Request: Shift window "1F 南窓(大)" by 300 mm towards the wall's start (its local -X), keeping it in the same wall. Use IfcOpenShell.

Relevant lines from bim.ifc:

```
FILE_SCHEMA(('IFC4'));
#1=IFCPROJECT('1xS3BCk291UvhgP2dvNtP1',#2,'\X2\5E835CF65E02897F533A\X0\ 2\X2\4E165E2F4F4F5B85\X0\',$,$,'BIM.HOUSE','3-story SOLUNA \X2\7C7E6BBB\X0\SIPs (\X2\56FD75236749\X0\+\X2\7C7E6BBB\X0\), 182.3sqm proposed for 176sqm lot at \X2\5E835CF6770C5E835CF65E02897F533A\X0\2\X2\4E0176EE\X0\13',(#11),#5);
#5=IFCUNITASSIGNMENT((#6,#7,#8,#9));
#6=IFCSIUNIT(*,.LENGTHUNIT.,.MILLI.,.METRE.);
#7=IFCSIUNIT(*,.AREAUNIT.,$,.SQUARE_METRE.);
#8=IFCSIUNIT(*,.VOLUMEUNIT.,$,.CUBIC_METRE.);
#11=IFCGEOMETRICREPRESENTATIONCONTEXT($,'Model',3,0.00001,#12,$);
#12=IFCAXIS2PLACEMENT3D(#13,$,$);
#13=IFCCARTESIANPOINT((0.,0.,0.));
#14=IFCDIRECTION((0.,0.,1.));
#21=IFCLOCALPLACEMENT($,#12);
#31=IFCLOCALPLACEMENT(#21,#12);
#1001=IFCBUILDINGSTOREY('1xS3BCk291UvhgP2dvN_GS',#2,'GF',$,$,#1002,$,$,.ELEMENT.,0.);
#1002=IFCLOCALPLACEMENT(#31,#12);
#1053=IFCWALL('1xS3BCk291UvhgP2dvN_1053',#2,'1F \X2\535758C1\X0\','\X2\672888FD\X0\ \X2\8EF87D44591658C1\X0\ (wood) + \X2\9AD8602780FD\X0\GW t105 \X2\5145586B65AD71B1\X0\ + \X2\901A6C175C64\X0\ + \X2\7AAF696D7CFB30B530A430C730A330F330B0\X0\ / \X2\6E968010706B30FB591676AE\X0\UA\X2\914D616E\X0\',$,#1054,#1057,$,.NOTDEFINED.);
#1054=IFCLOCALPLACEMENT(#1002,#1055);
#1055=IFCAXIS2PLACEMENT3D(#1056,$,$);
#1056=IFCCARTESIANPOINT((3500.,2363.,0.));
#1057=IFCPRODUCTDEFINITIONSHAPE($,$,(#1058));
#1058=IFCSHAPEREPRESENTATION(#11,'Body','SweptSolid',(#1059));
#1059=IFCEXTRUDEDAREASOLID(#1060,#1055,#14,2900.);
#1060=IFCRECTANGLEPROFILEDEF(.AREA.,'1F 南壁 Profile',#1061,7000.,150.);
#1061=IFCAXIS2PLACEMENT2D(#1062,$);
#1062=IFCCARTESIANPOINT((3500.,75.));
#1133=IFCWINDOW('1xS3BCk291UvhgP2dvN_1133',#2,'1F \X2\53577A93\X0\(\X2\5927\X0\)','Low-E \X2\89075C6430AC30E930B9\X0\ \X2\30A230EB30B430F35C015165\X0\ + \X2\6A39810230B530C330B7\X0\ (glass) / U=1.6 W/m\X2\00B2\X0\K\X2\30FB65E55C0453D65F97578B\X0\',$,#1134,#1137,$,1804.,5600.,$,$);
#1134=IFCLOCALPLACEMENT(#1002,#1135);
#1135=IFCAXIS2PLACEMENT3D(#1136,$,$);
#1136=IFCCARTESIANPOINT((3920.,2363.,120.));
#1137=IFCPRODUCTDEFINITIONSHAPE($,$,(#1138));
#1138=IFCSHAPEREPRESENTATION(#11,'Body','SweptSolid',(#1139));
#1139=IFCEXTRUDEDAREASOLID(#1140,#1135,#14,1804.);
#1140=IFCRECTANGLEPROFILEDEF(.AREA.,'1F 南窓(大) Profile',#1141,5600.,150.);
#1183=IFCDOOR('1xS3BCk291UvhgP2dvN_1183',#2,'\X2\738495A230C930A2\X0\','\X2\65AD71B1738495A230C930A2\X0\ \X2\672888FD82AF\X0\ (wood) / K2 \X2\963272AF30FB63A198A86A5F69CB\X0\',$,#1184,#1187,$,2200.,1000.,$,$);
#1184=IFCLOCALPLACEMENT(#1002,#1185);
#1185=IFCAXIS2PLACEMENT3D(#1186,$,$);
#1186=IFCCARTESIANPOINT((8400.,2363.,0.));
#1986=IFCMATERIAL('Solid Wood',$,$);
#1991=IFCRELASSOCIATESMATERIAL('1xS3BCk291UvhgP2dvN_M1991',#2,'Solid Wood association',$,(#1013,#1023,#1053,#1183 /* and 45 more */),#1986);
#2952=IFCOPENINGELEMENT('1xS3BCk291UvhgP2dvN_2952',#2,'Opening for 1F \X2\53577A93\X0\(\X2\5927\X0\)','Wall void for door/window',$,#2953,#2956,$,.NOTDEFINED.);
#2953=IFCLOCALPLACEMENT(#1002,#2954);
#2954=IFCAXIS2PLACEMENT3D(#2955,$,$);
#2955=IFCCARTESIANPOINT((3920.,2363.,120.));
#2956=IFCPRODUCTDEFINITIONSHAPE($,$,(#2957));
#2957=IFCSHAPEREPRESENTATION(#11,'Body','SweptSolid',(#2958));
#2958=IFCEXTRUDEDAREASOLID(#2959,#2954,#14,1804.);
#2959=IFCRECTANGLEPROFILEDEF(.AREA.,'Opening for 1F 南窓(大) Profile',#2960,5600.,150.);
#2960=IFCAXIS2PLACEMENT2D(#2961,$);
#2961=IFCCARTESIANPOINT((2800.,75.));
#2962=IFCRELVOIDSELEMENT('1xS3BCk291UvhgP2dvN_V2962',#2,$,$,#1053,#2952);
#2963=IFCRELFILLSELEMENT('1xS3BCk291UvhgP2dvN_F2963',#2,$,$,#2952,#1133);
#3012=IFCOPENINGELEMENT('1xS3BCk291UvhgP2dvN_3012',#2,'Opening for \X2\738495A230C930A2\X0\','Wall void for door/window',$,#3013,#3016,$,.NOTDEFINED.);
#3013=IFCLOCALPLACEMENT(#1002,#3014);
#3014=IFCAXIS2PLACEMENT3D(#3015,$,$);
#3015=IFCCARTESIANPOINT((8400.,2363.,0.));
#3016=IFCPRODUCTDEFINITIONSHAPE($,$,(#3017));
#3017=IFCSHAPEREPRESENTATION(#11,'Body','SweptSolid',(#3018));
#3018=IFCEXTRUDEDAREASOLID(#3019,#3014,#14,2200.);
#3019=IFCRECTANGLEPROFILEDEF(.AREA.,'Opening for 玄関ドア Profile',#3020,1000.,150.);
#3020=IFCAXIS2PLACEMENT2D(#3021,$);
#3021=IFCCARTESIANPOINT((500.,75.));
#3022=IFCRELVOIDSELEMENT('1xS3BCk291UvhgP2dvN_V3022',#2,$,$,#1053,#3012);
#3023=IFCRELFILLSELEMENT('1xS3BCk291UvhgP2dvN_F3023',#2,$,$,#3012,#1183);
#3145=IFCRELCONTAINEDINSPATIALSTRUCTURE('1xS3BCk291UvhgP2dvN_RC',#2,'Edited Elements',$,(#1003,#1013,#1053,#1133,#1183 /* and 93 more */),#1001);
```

```python
import ifcopenshell
import ifcopenshell.api.geometry
import ifcopenshell.util.placement

model = ifcopenshell.open("bim.ifc")

window = model.by_guid("1xS3BCk291UvhgP2dvN_1133")
opening = window.FillsVoids[0].RelatingOpeningElement
wall = opening.VoidsElements[0].RelatingBuildingElement

wall_matrix = ifcopenshell.util.placement.get_local_placement(wall.ObjectPlacement)
shift = wall_matrix[:3, 0] * -300.0
before = ifcopenshell.util.placement.get_local_placement(window.ObjectPlacement)[:3, 3].copy()

# The window is not placed relative to its opening, so move both.
for product in (opening, window):
    matrix = ifcopenshell.util.placement.get_local_placement(product.ObjectPlacement)
    matrix[:3, 3] += shift
    ifcopenshell.api.geometry.edit_object_placement(model, product=product, matrix=matrix, is_si=False)

after = ifcopenshell.util.placement.get_local_placement(window.ObjectPlacement)[:3, 3]
print("window moved by", (after - before).round(3) + 0.0)

model.write("bim_edited.ifc")
```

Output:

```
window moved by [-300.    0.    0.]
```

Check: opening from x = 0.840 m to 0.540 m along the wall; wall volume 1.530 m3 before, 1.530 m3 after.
